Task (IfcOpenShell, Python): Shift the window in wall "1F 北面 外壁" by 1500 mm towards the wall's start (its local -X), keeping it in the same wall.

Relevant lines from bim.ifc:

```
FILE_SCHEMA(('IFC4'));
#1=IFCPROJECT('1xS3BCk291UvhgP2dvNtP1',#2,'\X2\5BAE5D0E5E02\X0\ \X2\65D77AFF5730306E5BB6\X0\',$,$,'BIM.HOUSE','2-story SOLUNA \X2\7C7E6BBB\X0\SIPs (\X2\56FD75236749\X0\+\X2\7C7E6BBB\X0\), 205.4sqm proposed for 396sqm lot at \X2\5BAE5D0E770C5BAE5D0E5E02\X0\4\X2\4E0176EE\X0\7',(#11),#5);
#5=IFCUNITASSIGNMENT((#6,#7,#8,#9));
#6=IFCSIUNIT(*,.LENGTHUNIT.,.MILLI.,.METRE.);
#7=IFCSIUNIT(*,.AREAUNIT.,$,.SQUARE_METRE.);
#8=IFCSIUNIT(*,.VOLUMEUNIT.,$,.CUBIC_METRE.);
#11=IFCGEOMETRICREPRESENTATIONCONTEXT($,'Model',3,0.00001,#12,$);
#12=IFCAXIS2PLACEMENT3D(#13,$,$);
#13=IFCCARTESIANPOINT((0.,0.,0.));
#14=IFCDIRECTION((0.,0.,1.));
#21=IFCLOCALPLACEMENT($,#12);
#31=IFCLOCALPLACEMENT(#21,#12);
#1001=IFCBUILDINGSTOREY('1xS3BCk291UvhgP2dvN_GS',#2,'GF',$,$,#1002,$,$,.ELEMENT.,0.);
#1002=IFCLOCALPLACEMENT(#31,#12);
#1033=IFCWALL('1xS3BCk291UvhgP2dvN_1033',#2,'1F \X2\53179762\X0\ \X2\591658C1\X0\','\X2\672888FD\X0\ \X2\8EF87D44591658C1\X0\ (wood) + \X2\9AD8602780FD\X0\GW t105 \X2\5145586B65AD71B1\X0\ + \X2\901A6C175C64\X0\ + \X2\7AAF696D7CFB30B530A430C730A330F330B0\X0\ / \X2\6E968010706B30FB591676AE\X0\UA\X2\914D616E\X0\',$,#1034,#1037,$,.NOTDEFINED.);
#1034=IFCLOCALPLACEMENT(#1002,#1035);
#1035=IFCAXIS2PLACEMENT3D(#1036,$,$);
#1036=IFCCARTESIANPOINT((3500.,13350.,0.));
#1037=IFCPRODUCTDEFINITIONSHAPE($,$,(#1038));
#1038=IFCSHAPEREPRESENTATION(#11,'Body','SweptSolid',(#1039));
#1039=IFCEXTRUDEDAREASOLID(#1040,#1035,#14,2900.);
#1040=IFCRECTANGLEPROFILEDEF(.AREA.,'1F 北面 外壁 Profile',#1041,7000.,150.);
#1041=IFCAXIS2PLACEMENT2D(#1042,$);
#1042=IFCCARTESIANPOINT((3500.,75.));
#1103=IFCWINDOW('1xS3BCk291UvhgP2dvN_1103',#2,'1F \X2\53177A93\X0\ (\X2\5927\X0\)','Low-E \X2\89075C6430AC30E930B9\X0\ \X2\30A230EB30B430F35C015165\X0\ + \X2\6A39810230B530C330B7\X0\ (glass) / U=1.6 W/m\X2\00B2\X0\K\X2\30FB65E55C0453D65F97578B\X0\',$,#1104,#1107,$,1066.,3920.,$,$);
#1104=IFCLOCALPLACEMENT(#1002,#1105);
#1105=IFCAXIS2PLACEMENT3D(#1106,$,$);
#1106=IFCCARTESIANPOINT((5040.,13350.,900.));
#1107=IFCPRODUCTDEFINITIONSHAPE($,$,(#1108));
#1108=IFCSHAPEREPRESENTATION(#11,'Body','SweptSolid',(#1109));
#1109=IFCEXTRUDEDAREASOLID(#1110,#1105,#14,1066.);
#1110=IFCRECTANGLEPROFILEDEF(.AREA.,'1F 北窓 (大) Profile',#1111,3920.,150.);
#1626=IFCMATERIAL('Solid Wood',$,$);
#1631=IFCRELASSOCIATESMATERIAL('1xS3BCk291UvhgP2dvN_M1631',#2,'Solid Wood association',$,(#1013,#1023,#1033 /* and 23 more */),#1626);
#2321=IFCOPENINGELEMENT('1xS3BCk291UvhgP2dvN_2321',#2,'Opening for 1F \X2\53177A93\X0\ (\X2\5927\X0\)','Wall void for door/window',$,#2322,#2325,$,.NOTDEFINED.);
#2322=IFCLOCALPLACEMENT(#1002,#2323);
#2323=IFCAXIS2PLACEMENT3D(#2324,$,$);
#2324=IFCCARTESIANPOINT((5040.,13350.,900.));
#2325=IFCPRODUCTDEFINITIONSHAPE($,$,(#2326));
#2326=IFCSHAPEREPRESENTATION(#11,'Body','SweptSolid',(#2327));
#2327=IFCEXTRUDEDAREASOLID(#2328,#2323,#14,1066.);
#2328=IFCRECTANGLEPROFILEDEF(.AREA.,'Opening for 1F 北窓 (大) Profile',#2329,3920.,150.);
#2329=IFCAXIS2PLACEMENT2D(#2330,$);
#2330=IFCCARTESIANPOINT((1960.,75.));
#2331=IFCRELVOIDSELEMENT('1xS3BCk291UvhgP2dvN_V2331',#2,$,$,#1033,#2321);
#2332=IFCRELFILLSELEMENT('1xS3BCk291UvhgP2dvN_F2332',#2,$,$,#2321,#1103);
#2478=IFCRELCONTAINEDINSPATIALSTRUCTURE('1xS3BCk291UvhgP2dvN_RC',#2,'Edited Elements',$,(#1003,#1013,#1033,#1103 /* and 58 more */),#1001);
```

```python
import ifcopenshell
import ifcopenshell.api.geometry
import ifcopenshell.util.placement
import ifcopenshell.util.unit

model = ifcopenshell.open("bim.ifc")
unit_scale = ifcopenshell.util.unit.calculate_unit_scale(model)

window = model.by_guid("1xS3BCk291UvhgP2dvN_1103")
opening = window.FillsVoids[0].RelatingOpeningElement
wall = opening.VoidsElements[0].RelatingBuildingElement

wall_matrix = ifcopenshell.util.placement.get_local_placement(wall.ObjectPlacement)
shift = wall_matrix[:3, 0] * -1.5 / unit_scale
before = ifcopenshell.util.placement.get_local_placement(window.ObjectPlacement)[:3, 3].copy()

# The window is not placed relative to its opening, so move both.
for product in (opening, window):
    matrix = ifcopenshell.util.placement.get_local_placement(product.ObjectPlacement)
    matrix[:3, 3] += shift
    ifcopenshell.api.geometry.edit_object_placement(model, product=product, matrix=matrix, is_si=False)

after = ifcopenshell.util.placement.get_local_placement(window.ObjectPlacement)[:3, 3]
print("window moved by", (after - before).round(3) + 0.0)

model.write("bim_edited.ifc")
```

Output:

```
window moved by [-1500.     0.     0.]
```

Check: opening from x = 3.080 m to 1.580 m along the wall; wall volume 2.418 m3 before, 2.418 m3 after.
